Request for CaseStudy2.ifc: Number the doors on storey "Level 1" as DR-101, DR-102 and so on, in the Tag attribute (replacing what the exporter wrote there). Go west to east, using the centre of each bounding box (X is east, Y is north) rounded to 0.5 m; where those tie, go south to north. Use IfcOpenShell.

First a look at what the model holds.

```python
import ifcopenshell
import ifcopenshell.util.element
import ifcopenshell.util.placement

model = ifcopenshell.open("CaseStudy2.ifc")
print(model.schema)
storey = next(s for s in model.by_type("IfcBuildingStorey") if s.Name == "Level 1")
doors = [e for e in ifcopenshell.util.element.get_decomposition(storey) if e.is_a("IfcDoor")]
for e in sorted(doors, key=lambda e: e.id()):
    origin = ifcopenshell.util.placement.get_local_placement(e.ObjectPlacement)[:3, 3]
    print(e.id(), e.Tag, e.Name, origin.round(2) + 0.0, sep=" | ")
```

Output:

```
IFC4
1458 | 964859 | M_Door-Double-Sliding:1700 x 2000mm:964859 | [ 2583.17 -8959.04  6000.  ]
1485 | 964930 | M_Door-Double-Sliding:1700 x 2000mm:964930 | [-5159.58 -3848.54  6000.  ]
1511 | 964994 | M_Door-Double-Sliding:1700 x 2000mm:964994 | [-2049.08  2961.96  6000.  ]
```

```python
import ifcopenshell
import ifcopenshell.geom
import ifcopenshell.util.element
import ifcopenshell.util.shape

model = ifcopenshell.open("CaseStudy2.ifc")
settings = ifcopenshell.geom.settings()
settings.set("use-world-coords", True)


def centre(element):
    shape = ifcopenshell.geom.create_shape(settings, element)
    return ifcopenshell.util.shape.get_bbox_centroid(shape.geometry)


storey = next(s for s in model.by_type("IfcBuildingStorey") if s.Name == "Level 1")
doors = [e for e in ifcopenshell.util.element.get_decomposition(storey) if e.is_a("IfcDoor")]

# Insertion points can sit at a corner or the storey origin, so sort by the geometry (in metres).
centres = {e: centre(e) for e in doors}
doors.sort(key=lambda e: (round(centres[e][0] / 0.5), centres[e][1]))

for i, e in enumerate(doors, start=1):
    number = f"DR-1{i:02d}"
    e.Tag = number
    print(e.id(), number)

model.write("CaseStudy2_updated.ifc")
```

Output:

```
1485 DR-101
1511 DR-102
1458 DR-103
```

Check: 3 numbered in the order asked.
